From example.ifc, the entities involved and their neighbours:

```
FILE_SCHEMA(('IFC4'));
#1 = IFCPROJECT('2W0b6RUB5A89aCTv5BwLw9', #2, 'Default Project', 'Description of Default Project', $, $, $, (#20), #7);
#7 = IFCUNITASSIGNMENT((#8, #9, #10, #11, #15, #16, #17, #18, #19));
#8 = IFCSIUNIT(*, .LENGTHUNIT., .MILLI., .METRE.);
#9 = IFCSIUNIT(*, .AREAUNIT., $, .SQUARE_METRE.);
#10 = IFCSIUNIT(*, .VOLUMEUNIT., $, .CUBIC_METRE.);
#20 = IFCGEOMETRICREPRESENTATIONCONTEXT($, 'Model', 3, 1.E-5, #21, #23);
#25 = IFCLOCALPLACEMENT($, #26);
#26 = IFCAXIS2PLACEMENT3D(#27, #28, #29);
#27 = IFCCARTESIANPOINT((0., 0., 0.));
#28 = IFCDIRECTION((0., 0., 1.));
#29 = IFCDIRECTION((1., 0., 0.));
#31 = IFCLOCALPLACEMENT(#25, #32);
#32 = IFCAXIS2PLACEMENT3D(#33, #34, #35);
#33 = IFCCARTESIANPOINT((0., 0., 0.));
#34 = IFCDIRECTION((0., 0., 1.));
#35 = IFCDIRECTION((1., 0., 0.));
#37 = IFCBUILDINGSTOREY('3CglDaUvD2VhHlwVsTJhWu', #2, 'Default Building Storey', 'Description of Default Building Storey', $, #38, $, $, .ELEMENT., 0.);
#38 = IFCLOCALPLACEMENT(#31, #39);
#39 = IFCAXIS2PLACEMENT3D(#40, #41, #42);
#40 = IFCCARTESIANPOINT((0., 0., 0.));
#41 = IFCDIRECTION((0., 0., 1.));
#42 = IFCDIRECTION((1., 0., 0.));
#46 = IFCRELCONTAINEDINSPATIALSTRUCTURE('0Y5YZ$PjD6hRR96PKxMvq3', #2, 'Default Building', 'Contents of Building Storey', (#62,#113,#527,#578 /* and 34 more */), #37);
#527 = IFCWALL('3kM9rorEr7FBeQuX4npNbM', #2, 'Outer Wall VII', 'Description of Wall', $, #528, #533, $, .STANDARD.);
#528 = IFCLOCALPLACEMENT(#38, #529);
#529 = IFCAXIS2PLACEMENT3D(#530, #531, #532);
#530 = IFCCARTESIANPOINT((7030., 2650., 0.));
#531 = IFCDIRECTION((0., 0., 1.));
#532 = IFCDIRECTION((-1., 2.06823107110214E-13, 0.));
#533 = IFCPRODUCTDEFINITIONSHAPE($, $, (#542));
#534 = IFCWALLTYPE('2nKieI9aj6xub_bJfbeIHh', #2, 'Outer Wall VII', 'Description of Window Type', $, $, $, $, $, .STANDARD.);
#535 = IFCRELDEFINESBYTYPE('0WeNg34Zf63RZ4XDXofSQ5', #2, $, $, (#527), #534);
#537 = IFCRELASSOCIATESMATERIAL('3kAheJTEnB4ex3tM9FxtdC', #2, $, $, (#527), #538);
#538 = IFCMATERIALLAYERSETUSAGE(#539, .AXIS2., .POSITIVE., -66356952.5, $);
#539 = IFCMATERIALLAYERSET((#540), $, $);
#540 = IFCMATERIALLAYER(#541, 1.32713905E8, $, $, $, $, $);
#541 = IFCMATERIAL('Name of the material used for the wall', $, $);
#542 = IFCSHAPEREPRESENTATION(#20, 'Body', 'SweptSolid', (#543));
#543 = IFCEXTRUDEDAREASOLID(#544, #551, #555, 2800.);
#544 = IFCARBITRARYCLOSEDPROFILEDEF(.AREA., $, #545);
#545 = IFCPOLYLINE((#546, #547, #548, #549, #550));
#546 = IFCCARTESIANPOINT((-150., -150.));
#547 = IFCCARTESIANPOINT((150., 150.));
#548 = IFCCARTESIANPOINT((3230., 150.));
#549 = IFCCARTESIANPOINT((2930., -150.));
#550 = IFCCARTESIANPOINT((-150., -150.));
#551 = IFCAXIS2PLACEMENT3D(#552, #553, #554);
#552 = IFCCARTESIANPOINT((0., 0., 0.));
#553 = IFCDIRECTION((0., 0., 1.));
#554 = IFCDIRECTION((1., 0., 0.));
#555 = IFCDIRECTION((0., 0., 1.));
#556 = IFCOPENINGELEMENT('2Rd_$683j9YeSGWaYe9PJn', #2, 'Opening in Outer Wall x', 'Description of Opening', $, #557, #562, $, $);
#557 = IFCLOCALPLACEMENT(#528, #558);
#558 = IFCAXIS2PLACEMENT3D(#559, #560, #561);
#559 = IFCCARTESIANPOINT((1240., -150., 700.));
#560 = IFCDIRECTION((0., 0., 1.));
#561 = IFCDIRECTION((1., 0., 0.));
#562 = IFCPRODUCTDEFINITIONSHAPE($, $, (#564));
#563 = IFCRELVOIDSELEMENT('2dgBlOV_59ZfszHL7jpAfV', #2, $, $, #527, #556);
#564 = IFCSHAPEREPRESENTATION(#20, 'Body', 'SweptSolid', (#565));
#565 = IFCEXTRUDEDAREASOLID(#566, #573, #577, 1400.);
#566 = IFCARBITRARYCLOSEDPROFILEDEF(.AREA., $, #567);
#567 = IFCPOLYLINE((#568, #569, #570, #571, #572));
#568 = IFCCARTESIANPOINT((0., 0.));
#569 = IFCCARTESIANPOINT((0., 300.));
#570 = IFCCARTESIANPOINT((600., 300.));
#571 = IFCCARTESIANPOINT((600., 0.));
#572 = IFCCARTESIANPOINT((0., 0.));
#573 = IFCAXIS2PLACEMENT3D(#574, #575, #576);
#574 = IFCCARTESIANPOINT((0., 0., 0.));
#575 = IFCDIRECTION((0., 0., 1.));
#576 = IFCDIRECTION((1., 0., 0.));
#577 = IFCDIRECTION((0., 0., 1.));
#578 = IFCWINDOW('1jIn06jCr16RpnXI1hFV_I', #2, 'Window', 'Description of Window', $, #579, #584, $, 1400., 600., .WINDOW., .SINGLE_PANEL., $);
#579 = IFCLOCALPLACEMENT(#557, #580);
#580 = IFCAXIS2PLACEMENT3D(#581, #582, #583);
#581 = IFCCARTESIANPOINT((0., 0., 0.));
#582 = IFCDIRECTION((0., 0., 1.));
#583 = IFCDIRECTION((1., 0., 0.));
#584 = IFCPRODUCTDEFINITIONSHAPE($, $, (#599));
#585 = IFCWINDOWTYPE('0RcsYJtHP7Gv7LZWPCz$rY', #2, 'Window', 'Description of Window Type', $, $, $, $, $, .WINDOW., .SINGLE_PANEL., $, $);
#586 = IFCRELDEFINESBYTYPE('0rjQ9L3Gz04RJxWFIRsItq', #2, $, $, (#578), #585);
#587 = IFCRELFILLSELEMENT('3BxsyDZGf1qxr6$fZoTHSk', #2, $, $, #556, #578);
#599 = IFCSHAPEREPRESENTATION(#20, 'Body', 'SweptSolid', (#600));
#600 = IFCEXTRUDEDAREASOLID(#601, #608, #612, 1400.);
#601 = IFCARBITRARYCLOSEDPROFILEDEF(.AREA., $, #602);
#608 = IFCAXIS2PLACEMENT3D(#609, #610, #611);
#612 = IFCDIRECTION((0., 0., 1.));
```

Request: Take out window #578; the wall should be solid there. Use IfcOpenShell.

```python
import ifcopenshell
import ifcopenshell.api.feature
import ifcopenshell.api.root
import ifcopenshell.geom
import ifcopenshell.util.shape

model = ifcopenshell.open("example.ifc")
settings = ifcopenshell.geom.settings()


def volume(element):
    """Net volume in cubic metres, openings subtracted."""
    shape = ifcopenshell.geom.create_shape(settings, element)
    return ifcopenshell.util.shape.get_volume(shape.geometry)


window = model.by_guid("1jIn06jCr16RpnXI1hFV_I")
opening = window.FillsVoids[0].RelatingOpeningElement
wall = opening.VoidsElements[0].RelatingBuildingElement
before = volume(wall)

ifcopenshell.api.root.remove_product(model, product=window)
ifcopenshell.api.feature.remove_feature(model, feature=opening)

after = volume(wall)

print(f"wall volume {before:.3f} -> {after:.3f} m3")

model.write("example-out.ifc")
```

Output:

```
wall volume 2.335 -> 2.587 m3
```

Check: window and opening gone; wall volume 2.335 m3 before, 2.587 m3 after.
